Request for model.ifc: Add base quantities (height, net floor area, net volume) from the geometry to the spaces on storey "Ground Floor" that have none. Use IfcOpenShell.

First a look at what the model holds.

```python
import ifcopenshell
import ifcopenshell.util.element
import ifcopenshell.util.unit

model = ifcopenshell.open("model.ifc")
print(model.schema)
for unit_type in ("LENGTHUNIT", "AREAUNIT", "VOLUMEUNIT"):
    print(unit_type, ifcopenshell.util.unit.calculate_unit_scale(model, unit_type))
storey = next(s for s in model.by_type("IfcBuildingStorey") if s.Name == "Ground Floor")
spaces = [e for e in ifcopenshell.util.element.get_decomposition(storey) if e.is_a("IfcSpace")]
for e in sorted(spaces, key=lambda e: e.id()):
    print(e.id(), e.is_a(), e.Name, list(ifcopenshell.util.element.get_psets(e, qtos_only=True)), sep=" | ")
```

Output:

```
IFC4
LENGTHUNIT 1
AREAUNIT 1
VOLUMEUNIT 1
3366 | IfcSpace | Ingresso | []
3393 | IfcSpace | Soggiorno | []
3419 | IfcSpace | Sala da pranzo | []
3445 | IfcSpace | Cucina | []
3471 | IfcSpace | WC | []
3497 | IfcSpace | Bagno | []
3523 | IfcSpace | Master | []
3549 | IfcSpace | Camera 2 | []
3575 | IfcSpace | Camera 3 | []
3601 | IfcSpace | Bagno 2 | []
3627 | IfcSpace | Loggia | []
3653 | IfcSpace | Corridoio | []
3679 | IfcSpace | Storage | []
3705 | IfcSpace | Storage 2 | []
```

```python
import ifcopenshell
import ifcopenshell.api.pset
import ifcopenshell.geom
import ifcopenshell.util.element
import ifcopenshell.util.shape
import ifcopenshell.util.unit

model = ifcopenshell.open("model.ifc")
unit_scale = ifcopenshell.util.unit.calculate_unit_scale(model)
area_scale = ifcopenshell.util.unit.calculate_unit_scale(model, "AREAUNIT")
volume_scale = ifcopenshell.util.unit.calculate_unit_scale(model, "VOLUMEUNIT")
settings = ifcopenshell.geom.settings()

storey = next(s for s in model.by_type("IfcBuildingStorey") if s.Name == "Ground Floor")
spaces = [e for e in ifcopenshell.util.element.get_decomposition(storey) if e.is_a("IfcSpace")]

for e in sorted(spaces, key=lambda e: e.id()):
    if ifcopenshell.util.element.get_psets(e, qtos_only=True, should_inherit=False):
        continue
    # Geometry comes back in metres, in the element's own axes.
    shape = ifcopenshell.geom.create_shape(settings, e)
    values = {
        "Height": ifcopenshell.util.shape.get_z(shape.geometry) / unit_scale,
        "NetFloorArea": ifcopenshell.util.shape.get_footprint_area(shape.geometry) / area_scale,
        "NetVolume": ifcopenshell.util.shape.get_volume(shape.geometry) / volume_scale,
    }
    qto = ifcopenshell.api.pset.add_qto(model, product=e, name="Qto_SpaceBaseQuantities")
    ifcopenshell.api.pset.edit_qto(model, qto=qto, properties=values)
    print(e.id(), {k: round(v, 3) for k, v in values.items()})

model.write("model_edited.ifc")
```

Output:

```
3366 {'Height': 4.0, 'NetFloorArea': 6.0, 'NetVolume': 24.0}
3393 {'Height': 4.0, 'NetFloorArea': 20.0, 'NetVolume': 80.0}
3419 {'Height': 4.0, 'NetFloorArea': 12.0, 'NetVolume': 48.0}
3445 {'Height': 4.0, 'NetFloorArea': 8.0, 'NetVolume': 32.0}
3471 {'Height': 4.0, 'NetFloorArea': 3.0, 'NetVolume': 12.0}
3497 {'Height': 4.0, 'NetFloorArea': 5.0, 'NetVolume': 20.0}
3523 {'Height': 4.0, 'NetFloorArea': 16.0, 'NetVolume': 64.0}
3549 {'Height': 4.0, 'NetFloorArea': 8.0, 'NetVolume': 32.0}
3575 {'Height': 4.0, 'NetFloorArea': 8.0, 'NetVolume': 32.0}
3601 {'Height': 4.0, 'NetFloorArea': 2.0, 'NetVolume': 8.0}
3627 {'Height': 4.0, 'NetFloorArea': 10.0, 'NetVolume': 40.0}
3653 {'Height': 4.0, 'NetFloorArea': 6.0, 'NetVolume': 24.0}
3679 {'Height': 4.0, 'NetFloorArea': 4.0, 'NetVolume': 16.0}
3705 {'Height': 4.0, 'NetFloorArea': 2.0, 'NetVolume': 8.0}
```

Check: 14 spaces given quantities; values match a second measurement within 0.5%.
